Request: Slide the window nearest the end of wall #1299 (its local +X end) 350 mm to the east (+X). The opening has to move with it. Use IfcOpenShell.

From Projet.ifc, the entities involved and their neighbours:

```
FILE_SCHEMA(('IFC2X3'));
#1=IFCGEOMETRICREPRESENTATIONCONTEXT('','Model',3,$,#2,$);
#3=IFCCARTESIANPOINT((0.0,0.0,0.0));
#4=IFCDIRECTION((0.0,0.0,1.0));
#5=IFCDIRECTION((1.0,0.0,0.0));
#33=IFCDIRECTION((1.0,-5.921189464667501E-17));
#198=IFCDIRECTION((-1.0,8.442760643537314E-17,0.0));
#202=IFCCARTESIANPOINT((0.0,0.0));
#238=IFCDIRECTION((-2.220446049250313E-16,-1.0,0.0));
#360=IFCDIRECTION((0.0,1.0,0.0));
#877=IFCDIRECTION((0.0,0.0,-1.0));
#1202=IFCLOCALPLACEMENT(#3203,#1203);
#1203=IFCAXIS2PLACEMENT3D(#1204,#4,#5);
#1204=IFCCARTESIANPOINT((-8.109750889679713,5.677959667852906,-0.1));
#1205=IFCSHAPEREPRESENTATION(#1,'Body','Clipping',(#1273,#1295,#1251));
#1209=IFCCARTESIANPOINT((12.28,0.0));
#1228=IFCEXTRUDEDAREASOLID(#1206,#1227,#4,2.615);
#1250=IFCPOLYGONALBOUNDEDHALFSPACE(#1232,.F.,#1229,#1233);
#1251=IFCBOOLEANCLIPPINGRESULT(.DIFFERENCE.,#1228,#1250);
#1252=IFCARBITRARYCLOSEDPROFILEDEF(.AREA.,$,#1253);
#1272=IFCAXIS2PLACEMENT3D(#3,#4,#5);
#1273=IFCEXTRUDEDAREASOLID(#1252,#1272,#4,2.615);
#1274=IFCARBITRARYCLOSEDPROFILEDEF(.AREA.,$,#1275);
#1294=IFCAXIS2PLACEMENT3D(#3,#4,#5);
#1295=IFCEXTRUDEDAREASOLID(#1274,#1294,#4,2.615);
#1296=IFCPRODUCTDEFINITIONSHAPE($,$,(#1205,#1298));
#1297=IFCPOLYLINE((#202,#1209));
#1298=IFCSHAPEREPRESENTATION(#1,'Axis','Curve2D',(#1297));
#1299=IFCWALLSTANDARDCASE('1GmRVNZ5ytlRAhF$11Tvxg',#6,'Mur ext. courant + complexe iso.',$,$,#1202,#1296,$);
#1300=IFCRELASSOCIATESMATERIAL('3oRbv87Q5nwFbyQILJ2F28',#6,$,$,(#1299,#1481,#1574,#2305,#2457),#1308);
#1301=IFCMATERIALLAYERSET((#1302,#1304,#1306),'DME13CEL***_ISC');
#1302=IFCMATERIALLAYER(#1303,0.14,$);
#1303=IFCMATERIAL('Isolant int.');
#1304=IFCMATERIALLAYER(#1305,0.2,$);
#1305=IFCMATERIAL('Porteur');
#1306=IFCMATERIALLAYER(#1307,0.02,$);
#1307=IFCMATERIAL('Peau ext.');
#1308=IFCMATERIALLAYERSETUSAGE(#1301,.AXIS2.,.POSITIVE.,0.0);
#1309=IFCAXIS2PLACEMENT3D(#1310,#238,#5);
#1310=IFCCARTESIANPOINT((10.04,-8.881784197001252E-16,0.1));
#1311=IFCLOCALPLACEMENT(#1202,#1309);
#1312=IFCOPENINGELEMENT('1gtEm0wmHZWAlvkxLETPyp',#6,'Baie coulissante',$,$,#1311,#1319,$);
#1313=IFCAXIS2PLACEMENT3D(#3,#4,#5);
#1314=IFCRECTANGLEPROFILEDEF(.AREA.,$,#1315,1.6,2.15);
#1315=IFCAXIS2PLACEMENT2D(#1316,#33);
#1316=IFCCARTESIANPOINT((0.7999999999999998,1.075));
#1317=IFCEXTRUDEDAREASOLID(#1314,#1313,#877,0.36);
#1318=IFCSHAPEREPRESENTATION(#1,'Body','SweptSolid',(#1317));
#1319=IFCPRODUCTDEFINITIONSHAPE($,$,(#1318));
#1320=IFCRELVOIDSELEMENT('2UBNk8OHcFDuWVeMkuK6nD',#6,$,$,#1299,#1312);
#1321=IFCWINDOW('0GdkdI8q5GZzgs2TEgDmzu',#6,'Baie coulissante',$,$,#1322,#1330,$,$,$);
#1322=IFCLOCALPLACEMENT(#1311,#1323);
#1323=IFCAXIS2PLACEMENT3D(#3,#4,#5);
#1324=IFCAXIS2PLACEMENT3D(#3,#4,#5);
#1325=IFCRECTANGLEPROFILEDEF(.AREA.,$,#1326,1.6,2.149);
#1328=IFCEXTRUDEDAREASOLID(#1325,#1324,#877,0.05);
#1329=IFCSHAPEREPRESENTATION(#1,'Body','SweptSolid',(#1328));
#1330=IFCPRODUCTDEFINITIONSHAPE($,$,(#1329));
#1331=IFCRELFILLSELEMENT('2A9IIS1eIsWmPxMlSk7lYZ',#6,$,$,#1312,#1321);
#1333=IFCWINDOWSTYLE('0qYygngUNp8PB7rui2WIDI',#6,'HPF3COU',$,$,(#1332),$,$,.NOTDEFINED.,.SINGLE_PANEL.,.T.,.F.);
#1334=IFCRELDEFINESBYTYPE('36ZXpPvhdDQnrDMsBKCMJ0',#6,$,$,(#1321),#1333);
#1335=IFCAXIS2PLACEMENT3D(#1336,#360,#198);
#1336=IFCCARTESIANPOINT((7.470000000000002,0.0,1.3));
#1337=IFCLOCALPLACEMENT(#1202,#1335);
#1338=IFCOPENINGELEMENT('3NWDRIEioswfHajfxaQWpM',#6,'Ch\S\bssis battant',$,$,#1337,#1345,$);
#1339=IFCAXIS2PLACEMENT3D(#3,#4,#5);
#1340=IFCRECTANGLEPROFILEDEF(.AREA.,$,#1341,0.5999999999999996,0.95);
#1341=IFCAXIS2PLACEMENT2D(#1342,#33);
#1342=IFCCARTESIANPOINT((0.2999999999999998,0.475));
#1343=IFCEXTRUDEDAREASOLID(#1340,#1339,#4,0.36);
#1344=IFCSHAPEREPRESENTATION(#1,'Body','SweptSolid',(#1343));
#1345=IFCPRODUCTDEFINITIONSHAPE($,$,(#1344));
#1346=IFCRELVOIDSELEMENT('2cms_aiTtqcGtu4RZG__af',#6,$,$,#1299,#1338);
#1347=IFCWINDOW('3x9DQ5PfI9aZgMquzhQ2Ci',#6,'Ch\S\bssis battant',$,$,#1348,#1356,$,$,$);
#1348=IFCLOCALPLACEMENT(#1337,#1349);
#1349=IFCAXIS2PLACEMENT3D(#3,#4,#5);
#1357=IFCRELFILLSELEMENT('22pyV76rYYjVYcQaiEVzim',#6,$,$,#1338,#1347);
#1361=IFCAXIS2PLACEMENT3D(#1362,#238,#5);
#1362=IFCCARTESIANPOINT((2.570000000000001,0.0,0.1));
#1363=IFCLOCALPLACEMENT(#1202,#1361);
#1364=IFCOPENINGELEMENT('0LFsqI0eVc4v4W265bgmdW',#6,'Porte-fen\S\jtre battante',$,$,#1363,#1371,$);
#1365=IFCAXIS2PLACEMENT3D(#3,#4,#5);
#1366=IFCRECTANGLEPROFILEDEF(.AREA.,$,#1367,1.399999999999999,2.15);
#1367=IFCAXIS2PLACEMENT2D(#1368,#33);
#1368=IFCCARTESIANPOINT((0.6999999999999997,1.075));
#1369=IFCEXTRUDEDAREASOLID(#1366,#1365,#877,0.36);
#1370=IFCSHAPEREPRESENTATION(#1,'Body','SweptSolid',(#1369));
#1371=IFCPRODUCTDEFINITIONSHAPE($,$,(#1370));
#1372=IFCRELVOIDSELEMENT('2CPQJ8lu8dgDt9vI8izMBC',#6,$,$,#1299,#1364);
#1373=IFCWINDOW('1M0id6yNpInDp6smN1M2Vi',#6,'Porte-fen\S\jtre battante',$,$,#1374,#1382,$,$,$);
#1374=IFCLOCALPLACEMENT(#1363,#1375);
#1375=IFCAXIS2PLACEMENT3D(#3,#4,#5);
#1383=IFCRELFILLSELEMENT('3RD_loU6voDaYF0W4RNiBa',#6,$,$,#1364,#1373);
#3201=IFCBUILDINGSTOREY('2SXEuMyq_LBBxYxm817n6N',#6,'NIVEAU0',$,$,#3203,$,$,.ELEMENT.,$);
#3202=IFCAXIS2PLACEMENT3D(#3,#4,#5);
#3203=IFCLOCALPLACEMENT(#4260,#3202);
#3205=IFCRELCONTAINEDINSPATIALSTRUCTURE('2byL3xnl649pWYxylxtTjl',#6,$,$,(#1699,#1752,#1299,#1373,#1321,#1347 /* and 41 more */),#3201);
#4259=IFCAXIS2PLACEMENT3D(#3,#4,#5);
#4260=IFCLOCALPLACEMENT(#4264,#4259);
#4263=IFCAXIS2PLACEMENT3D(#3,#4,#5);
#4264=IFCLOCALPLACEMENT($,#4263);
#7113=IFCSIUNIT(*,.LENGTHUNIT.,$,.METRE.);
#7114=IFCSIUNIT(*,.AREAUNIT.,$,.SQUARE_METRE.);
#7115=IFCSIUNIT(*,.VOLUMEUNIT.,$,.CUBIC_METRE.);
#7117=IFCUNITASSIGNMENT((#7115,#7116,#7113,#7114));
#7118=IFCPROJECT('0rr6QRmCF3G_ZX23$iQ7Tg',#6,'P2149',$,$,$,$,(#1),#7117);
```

```python
import ifcopenshell
import ifcopenshell.api.geometry
import ifcopenshell.util.placement
import ifcopenshell.util.unit

model = ifcopenshell.open("Projet.ifc")
unit_scale = ifcopenshell.util.unit.calculate_unit_scale(model)

window = model.by_guid("0GdkdI8q5GZzgs2TEgDmzu")
opening = window.FillsVoids[0].RelatingOpeningElement
wall = opening.VoidsElements[0].RelatingBuildingElement

wall_matrix = ifcopenshell.util.placement.get_local_placement(wall.ObjectPlacement)
shift = wall_matrix[:3, 0] * 0.35 / unit_scale
before = ifcopenshell.util.placement.get_local_placement(window.ObjectPlacement)[:3, 3].copy()

# The window is placed relative to its opening, so it follows when the opening moves.
matrix = ifcopenshell.util.placement.get_local_placement(opening.ObjectPlacement)
matrix[:3, 3] += shift
ifcopenshell.api.geometry.edit_object_placement(
    model, product=opening, matrix=matrix, is_si=False, should_transform_children=True
)

after = ifcopenshell.util.placement.get_local_placement(window.ObjectPlacement)[:3, 3]
print("window moved by", (after - before).round(3) + 0.0)

model.write("Projet_rev.ifc")
```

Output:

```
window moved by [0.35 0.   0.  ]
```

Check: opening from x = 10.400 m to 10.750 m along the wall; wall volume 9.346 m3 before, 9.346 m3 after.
